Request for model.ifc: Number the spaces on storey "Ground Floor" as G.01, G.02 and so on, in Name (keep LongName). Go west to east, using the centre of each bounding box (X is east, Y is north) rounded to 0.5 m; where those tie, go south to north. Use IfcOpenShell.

First a look at what the model holds.

```python
import ifcopenshell
import ifcopenshell.util.element
import ifcopenshell.util.placement

model = ifcopenshell.open("model.ifc")
print(model.schema)
storey = next(s for s in model.by_type("IfcBuildingStorey") if s.Name == "Ground Floor")
spaces = [e for e in ifcopenshell.util.element.get_decomposition(storey) if e.is_a("IfcSpace")]
for e in sorted(spaces, key=lambda e: e.id()):
    origin = ifcopenshell.util.placement.get_local_placement(e.ObjectPlacement)[:3, 3]
    print(e.id(), e.Name, e.LongName, origin.round(2) + 0.0, sep=" | ")
```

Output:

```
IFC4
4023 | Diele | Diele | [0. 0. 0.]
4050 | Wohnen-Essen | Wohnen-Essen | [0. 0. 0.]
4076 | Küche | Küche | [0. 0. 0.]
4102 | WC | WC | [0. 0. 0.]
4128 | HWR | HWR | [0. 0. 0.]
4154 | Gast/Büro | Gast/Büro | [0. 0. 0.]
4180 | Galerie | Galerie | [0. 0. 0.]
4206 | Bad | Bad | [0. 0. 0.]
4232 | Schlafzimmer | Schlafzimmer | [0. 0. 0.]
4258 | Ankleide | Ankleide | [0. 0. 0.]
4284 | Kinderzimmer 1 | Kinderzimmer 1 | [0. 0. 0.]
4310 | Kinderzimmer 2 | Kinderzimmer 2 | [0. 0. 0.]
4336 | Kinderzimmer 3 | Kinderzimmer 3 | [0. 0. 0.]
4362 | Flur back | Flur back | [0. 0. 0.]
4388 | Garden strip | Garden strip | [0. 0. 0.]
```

```python
import ifcopenshell
import ifcopenshell.geom
import ifcopenshell.util.element
import ifcopenshell.util.shape

model = ifcopenshell.open("model.ifc")
settings = ifcopenshell.geom.settings()
settings.set("use-world-coords", True)


def centre(element):
    shape = ifcopenshell.geom.create_shape(settings, element)
    return ifcopenshell.util.shape.get_bbox_centroid(shape.geometry)


storey = next(s for s in model.by_type("IfcBuildingStorey") if s.Name == "Ground Floor")
spaces = [e for e in ifcopenshell.util.element.get_decomposition(storey) if e.is_a("IfcSpace")]

# Insertion points can sit at a corner or the storey origin, so sort by the geometry (in metres).
centres = {e: centre(e) for e in spaces}
spaces.sort(key=lambda e: (round(centres[e][0] / 0.5), centres[e][1]))

for i, e in enumerate(spaces, start=1):
    number = f"G.{i:02d}"
    e.Name = number
    print(e.id(), number)

model.write("model_edited.ifc")
```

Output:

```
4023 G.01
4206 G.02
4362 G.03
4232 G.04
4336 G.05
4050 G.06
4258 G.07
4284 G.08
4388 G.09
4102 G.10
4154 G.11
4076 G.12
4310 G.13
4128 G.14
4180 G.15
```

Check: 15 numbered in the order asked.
